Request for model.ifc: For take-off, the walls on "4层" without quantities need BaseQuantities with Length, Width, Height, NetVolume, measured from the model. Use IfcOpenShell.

First a look at what the model holds.

```python
import ifcopenshell
import ifcopenshell.util.element
import ifcopenshell.util.unit

model = ifcopenshell.open("model.ifc")
print(model.schema)
for unit_type in ("LENGTHUNIT", "AREAUNIT", "VOLUMEUNIT"):
    print(unit_type, ifcopenshell.util.unit.calculate_unit_scale(model, unit_type))
storey = next(s for s in model.by_type("IfcBuildingStorey") if s.Name == "4层")
walls = [e for e in ifcopenshell.util.element.get_decomposition(storey) if e.is_a("IfcWall")]
for e in sorted(walls, key=lambda e: e.id()):
    print(e.id(), e.is_a(), e.Name, list(ifcopenshell.util.element.get_psets(e, qtos_only=True)), sep=" | ")
```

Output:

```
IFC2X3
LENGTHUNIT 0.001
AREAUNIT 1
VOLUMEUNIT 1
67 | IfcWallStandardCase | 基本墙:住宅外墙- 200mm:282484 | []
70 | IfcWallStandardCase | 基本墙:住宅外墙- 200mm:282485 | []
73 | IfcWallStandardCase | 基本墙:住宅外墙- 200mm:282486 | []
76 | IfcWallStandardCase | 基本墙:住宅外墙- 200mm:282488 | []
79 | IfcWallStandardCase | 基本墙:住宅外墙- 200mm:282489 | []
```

```python
import ifcopenshell
import ifcopenshell.api.pset
import ifcopenshell.geom
import ifcopenshell.util.element
import ifcopenshell.util.shape
import ifcopenshell.util.unit

model = ifcopenshell.open("model.ifc")
unit_scale = ifcopenshell.util.unit.calculate_unit_scale(model)
volume_scale = ifcopenshell.util.unit.calculate_unit_scale(model, "VOLUMEUNIT")
settings = ifcopenshell.geom.settings()

storey = next(s for s in model.by_type("IfcBuildingStorey") if s.Name == "4层")
walls = [e for e in ifcopenshell.util.element.get_decomposition(storey) if e.is_a("IfcWall")]

for e in sorted(walls, key=lambda e: e.id()):
    if ifcopenshell.util.element.get_psets(e, qtos_only=True, should_inherit=False):
        continue
    # Geometry comes back in metres, in the element's own axes.
    shape = ifcopenshell.geom.create_shape(settings, e)
    values = {
        "Length": ifcopenshell.util.shape.get_x(shape.geometry) / unit_scale,
        "Width": ifcopenshell.util.shape.get_y(shape.geometry) / unit_scale,
        "Height": ifcopenshell.util.shape.get_z(shape.geometry) / unit_scale,
        "NetVolume": ifcopenshell.util.shape.get_volume(shape.geometry) / volume_scale,
    }
    qto = ifcopenshell.api.pset.add_qto(model, product=e, name="BaseQuantities")
    ifcopenshell.api.pset.edit_qto(model, qto=qto, properties=values)
    print(e.id(), {k: round(v, 3) for k, v in values.items()})

model.write("model-out.ifc")
```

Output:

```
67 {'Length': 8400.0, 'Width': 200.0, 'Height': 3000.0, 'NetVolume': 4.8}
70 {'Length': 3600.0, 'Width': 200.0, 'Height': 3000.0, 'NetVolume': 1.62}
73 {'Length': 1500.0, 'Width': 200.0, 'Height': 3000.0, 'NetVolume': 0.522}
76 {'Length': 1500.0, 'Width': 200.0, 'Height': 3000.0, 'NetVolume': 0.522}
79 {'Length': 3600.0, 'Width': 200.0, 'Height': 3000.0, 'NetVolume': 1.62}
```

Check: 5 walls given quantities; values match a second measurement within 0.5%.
